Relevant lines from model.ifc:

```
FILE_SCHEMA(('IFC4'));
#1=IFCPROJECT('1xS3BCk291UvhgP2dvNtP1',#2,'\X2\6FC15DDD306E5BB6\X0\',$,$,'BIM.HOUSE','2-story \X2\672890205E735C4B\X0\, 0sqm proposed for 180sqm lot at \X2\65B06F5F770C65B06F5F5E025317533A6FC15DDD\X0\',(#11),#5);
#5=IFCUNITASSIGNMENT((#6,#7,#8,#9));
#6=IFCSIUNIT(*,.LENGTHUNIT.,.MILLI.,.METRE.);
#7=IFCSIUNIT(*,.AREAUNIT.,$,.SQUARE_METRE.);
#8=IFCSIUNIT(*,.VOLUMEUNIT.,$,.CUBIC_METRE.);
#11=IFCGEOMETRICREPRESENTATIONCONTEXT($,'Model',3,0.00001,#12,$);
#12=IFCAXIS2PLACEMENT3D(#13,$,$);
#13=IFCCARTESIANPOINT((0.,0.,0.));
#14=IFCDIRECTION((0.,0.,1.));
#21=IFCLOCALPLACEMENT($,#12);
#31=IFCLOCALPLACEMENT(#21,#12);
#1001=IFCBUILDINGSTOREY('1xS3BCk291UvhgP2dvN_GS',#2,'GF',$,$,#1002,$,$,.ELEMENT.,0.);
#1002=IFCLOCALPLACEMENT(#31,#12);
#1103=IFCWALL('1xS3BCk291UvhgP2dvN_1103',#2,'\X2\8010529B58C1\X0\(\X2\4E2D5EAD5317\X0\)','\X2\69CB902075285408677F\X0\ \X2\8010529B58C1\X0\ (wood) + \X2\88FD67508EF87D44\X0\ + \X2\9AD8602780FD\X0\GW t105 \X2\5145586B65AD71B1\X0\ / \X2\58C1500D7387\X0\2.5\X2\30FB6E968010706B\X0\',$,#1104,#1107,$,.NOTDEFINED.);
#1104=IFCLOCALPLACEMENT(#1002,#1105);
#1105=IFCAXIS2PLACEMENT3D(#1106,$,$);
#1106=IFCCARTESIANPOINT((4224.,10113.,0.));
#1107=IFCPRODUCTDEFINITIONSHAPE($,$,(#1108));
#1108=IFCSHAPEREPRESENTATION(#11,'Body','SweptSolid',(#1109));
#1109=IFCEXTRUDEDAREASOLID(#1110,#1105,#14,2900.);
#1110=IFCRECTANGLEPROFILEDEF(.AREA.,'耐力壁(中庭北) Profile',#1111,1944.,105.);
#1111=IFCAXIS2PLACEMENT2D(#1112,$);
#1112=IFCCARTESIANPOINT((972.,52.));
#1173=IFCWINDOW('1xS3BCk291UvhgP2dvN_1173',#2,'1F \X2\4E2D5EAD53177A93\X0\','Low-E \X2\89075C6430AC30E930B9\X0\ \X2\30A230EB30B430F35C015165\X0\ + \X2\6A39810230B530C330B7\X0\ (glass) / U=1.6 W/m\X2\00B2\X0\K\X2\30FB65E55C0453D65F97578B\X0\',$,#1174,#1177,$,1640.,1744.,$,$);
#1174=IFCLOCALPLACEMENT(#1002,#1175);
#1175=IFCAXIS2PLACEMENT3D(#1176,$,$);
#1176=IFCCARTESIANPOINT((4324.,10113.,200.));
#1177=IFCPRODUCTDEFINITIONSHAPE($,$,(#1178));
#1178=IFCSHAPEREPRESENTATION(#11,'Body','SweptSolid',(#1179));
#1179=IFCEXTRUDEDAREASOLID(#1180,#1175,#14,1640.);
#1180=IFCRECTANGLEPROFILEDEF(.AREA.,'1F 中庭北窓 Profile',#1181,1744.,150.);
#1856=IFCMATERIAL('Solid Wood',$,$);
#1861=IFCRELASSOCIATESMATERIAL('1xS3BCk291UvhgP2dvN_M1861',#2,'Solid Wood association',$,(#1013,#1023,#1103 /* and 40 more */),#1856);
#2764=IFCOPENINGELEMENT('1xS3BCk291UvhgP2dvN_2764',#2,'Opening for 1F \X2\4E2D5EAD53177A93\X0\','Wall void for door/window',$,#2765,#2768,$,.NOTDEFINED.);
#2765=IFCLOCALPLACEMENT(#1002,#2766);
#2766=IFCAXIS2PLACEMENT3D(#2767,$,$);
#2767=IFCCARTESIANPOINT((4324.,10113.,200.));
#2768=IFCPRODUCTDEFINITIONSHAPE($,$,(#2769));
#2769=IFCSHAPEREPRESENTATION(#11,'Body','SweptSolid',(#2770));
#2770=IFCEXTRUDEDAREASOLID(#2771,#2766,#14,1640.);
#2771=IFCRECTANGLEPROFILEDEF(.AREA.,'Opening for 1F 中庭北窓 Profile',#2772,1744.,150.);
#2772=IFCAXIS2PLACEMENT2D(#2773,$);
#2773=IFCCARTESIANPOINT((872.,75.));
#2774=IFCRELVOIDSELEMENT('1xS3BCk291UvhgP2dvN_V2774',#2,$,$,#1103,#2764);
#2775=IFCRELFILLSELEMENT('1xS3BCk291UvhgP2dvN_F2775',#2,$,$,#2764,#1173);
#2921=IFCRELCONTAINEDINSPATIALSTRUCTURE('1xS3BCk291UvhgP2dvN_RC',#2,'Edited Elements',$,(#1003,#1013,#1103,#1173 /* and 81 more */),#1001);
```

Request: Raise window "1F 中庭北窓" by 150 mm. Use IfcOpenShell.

```python
import numpy as np
import ifcopenshell
import ifcopenshell.api.geometry
import ifcopenshell.util.placement
import ifcopenshell.util.unit

model = ifcopenshell.open("model.ifc")
unit_scale = ifcopenshell.util.unit.calculate_unit_scale(model)

window = model.by_guid("1xS3BCk291UvhgP2dvN_1173")
opening = window.FillsVoids[0].RelatingOpeningElement
dz = 150.0

shift = np.array([0.0, 0.0, dz])
# The window is not placed relative to its opening, so move both.
for product in (opening, window):
    matrix = ifcopenshell.util.placement.get_local_placement(product.ObjectPlacement)
    matrix[:3, 3] += shift
    ifcopenshell.api.geometry.edit_object_placement(model, product=product, matrix=matrix, is_si=False)

print(f"moved by {dz * unit_scale:+.3f} m")

model.write("model_rev.ifc")
```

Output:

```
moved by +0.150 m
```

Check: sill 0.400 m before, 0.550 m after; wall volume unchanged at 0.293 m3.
